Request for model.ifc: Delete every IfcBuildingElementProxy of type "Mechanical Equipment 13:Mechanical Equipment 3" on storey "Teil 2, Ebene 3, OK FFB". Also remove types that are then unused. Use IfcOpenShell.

First a look at what the model holds.

```python
import ifcopenshell
import ifcopenshell.util.element

model = ifcopenshell.open("model.ifc")
print(model.schema)
storey = next(s for s in model.by_type("IfcBuildingStorey") if s.Name == "Teil 2, Ebene 3, OK FFB")
proxies = [e for e in ifcopenshell.util.element.get_decomposition(storey) if e.is_a("IfcBuildingElementProxy")]
seen = {}
for e in proxies:
    element_type = ifcopenshell.util.element.get_type(e)
    name = element_type.Name if element_type not in (None, e) else None
    seen[name] = seen.get(name, 0) + 1
for name, count in sorted(seen.items(), key=str):
    print(count, "x", name)
```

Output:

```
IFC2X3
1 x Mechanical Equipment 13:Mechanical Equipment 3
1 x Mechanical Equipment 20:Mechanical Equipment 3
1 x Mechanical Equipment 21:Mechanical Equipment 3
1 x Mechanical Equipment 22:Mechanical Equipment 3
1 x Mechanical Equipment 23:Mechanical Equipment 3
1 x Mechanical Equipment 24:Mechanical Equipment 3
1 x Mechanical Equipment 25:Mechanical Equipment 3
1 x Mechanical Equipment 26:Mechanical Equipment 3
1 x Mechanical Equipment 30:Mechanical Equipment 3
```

```python
import ifcopenshell
import ifcopenshell.api.root
import ifcopenshell.util.element

model = ifcopenshell.open("model.ifc")

storey = next(s for s in model.by_type("IfcBuildingStorey") if s.Name == "Teil 2, Ebene 3, OK FFB")
proxies = [e for e in ifcopenshell.util.element.get_decomposition(storey) if e.is_a("IfcBuildingElementProxy")]
targets = [e for e in proxies if (t := ifcopenshell.util.element.get_type(e)) not in (None, e) and t.Name == "Mechanical Equipment 13:Mechanical Equipment 3"]
types = {ifcopenshell.util.element.get_type(e) for e in targets} - {None, *targets}

for e in targets:
    ifcopenshell.api.root.remove_product(model, product=e)
print(len(targets), "removed")

unused = [t for t in types if not ifcopenshell.util.element.get_types(t)]
for t in unused:
    ifcopenshell.api.root.remove_product(model, product=t)
print(len(unused), "unused types removed")

model.write("model_updated.ifc")
```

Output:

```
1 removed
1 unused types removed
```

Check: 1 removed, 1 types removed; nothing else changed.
